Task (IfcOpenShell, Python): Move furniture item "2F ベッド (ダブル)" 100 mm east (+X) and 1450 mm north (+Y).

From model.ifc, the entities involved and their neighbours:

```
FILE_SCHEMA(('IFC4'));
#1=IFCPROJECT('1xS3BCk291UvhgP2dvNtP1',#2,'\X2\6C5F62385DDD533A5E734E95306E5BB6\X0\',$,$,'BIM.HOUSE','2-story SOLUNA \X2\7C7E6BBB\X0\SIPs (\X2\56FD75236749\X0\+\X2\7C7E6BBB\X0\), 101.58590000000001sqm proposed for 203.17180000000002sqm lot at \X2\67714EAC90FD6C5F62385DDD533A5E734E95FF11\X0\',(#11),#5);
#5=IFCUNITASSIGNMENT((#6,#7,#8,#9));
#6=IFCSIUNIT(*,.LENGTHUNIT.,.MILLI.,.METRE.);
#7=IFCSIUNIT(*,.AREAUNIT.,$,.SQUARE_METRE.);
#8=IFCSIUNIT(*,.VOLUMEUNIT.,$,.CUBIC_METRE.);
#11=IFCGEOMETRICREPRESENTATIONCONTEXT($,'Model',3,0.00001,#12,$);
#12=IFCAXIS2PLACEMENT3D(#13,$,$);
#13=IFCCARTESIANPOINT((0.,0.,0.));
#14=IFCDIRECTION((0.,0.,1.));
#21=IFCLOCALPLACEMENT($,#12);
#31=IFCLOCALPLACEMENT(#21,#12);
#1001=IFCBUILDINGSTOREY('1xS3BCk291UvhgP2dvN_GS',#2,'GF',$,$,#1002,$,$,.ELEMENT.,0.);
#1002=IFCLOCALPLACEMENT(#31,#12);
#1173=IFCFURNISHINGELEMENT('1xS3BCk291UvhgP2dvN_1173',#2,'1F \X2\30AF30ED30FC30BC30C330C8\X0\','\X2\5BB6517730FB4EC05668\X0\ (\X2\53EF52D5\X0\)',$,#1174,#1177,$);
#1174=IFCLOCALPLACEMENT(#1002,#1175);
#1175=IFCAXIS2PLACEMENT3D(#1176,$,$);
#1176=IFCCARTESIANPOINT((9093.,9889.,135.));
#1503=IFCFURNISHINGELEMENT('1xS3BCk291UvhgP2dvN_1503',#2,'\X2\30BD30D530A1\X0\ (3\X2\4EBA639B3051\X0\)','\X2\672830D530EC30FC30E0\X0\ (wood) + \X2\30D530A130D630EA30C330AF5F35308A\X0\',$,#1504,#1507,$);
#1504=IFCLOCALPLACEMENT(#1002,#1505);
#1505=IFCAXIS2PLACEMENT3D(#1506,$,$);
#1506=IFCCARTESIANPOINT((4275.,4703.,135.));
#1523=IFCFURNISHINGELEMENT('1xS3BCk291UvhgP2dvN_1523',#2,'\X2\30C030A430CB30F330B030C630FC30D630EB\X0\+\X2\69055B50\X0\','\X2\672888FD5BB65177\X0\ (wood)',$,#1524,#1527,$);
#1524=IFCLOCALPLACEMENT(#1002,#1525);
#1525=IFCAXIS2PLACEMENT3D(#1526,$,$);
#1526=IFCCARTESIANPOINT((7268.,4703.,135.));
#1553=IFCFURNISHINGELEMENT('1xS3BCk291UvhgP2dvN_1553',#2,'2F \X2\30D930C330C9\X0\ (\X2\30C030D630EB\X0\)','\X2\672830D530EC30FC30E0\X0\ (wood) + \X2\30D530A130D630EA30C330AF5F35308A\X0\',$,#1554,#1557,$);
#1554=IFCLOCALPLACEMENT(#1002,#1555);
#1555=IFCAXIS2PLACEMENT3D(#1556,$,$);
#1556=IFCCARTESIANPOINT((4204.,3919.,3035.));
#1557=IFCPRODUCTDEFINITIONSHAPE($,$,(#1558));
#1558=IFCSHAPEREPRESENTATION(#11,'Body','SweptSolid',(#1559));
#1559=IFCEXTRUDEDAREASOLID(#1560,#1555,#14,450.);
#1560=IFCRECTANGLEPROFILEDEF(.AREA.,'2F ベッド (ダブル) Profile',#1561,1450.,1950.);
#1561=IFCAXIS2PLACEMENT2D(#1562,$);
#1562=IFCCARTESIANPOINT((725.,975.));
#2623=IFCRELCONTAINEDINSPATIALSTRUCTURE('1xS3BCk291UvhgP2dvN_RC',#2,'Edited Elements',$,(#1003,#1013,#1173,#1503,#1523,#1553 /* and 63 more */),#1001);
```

```python
import ifcopenshell
import ifcopenshell.api.geometry
import ifcopenshell.util.placement

model = ifcopenshell.open("model.ifc")

item = model.by_id(1553)
matrix = ifcopenshell.util.placement.get_local_placement(item.ObjectPlacement)
matrix[0, 3] += 100.0
matrix[1, 3] += 1450.0
ifcopenshell.api.geometry.edit_object_placement(model, product=item, matrix=matrix, is_si=False)

print(ifcopenshell.util.placement.get_local_placement(item.ObjectPlacement).round(3) + 0.0)

model.write("model_v2.ifc")
```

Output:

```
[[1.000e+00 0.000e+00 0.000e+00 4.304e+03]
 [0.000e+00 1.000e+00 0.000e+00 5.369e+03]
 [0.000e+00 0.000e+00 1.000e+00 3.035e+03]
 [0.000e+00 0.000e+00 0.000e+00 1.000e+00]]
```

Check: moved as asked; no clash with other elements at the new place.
